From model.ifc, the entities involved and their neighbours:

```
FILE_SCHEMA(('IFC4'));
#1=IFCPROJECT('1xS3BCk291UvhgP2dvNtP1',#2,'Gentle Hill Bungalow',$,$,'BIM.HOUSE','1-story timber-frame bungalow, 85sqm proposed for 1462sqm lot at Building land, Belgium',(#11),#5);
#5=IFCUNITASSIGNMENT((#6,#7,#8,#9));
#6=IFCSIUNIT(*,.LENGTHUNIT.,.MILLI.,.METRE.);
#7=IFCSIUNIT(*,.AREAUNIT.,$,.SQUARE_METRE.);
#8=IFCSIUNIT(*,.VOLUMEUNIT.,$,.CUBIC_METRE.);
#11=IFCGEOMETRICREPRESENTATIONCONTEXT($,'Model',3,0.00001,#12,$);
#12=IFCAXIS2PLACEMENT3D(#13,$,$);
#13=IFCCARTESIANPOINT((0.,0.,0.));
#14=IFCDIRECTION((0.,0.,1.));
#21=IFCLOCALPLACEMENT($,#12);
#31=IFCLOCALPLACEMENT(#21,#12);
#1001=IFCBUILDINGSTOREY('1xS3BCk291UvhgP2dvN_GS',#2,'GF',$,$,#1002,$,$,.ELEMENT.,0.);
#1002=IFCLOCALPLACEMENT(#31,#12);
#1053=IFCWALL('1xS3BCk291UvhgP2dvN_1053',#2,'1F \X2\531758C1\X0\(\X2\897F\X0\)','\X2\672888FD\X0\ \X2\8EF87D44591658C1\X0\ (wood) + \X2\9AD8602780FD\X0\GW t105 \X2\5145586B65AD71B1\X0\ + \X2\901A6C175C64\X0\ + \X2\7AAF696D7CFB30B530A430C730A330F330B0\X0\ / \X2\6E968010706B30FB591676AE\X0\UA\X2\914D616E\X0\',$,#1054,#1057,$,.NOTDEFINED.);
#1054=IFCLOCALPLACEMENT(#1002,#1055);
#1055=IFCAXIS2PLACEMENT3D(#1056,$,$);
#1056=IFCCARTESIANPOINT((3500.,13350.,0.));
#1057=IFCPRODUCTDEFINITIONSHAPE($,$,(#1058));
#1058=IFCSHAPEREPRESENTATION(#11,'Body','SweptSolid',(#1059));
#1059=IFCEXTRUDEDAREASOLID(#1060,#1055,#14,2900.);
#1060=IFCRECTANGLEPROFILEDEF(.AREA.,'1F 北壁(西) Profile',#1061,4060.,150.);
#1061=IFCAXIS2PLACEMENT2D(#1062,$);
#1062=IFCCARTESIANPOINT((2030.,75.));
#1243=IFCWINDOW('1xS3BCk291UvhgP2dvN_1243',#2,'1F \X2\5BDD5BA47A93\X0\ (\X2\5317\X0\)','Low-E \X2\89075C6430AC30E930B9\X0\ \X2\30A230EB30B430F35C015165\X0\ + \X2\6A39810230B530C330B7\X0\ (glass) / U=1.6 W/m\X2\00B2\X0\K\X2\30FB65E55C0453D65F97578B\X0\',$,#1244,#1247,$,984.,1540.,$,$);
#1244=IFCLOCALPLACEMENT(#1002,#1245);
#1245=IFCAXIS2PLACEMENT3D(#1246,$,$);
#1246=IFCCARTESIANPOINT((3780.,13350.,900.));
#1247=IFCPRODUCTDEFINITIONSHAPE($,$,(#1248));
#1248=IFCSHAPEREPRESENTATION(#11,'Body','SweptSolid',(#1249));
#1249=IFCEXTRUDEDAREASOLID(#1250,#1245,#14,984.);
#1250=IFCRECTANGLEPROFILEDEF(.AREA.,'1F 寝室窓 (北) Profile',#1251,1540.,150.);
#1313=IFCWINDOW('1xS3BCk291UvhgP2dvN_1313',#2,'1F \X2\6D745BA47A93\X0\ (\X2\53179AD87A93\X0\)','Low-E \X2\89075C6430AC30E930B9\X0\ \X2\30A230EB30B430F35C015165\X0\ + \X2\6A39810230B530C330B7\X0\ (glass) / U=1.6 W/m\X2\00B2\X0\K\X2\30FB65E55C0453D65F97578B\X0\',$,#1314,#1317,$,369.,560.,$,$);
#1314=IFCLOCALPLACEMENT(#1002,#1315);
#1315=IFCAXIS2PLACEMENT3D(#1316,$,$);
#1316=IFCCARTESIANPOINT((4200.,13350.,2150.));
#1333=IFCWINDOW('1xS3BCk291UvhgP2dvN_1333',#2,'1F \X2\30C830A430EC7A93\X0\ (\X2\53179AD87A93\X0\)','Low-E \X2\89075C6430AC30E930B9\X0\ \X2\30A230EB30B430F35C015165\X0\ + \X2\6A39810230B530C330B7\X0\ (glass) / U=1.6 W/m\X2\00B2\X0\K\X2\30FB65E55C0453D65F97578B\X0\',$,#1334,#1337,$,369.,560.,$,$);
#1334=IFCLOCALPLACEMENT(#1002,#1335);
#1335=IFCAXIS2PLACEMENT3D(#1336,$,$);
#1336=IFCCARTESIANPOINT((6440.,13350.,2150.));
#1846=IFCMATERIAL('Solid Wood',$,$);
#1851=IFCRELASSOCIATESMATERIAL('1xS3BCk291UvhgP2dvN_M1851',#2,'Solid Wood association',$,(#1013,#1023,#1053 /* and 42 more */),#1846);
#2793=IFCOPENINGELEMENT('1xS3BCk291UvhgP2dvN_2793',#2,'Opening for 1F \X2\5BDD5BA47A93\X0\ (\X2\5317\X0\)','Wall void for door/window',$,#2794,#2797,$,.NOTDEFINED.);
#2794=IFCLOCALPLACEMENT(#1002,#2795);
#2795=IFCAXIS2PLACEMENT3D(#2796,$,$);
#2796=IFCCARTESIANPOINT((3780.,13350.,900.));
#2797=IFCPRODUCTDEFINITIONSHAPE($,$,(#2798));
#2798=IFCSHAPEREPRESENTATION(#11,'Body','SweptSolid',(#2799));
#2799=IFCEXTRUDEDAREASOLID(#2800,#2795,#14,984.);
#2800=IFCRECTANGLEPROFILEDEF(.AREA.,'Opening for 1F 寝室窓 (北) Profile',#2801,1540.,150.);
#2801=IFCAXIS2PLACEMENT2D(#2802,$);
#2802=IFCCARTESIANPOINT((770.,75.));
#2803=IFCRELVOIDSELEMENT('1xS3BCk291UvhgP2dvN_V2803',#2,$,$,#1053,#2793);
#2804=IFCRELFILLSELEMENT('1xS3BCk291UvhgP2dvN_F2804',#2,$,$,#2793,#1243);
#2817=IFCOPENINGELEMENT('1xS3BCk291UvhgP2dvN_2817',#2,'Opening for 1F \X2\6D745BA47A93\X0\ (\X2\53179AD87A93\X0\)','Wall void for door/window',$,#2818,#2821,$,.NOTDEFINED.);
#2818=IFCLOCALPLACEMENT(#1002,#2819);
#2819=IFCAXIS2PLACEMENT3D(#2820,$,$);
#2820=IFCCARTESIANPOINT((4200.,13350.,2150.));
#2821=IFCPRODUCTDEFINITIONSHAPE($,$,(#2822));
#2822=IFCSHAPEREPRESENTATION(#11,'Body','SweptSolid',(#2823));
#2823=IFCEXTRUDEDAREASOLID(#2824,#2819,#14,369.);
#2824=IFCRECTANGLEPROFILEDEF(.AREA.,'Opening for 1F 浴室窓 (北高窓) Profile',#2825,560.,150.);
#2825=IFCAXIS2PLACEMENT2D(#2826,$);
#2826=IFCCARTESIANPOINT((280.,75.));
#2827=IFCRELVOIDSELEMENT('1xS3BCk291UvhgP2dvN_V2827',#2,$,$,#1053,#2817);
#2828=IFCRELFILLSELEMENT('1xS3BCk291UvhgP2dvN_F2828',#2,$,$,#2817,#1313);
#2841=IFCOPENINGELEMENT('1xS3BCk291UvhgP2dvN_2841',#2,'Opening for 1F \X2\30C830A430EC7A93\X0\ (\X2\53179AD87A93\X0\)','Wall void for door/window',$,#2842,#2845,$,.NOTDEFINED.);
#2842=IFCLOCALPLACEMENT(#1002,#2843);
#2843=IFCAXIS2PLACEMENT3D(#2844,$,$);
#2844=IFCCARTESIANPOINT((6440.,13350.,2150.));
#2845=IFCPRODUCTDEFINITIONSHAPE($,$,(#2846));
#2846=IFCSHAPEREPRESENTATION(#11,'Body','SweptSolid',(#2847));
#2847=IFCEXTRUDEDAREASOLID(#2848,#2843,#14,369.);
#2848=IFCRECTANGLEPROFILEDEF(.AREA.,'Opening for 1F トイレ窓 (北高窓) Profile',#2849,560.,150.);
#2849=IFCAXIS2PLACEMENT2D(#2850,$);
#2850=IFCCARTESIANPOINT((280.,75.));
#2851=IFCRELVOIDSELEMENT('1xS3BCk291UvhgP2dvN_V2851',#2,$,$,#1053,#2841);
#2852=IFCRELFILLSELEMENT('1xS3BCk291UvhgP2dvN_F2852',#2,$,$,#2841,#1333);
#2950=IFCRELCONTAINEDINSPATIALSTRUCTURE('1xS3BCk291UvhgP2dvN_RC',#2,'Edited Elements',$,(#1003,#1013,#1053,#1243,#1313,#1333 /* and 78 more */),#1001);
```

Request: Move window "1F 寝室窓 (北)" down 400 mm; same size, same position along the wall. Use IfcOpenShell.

```python
import numpy as np
import ifcopenshell
import ifcopenshell.api.geometry
import ifcopenshell.util.placement
import ifcopenshell.util.unit

model = ifcopenshell.open("model.ifc")
unit_scale = ifcopenshell.util.unit.calculate_unit_scale(model)

window = model.by_guid("1xS3BCk291UvhgP2dvN_1243")
opening = window.FillsVoids[0].RelatingOpeningElement
dz = -0.4 / unit_scale

shift = np.array([0.0, 0.0, dz])
# The window is not placed relative to its opening, so move both.
for product in (opening, window):
    matrix = ifcopenshell.util.placement.get_local_placement(product.ObjectPlacement)
    matrix[:3, 3] += shift
    ifcopenshell.api.geometry.edit_object_placement(model, product=product, matrix=matrix, is_si=False)

print(f"moved by {dz * unit_scale:+.3f} m")

model.write("model-out.ifc")
```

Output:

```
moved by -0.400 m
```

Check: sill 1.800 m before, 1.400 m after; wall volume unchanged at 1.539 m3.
